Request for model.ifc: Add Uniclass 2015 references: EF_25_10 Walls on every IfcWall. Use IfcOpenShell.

First a look at what the model holds.

```python
import ifcopenshell

model = ifcopenshell.open("model.ifc")
print(model.schema)
print("classifications:", [c.Name for c in model.by_type("IfcClassification")])
for ifc_class in ("IfcDoor", "IfcRoof", "IfcStair", "IfcWall", "IfcWindow"):
    print(ifc_class, len(model.by_type(ifc_class)))
```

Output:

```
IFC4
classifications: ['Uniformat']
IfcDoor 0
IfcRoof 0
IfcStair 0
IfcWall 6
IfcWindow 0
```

```python
import ifcopenshell
import ifcopenshell.api.classification

model = ifcopenshell.open("model.ifc")

system = ifcopenshell.api.classification.add_classification(model, classification="Uniclass 2015")

codes = {
    "IfcWall": ("EF_25_10", "Walls"),
}
for ifc_class, (code, name) in codes.items():
    products = model.by_type(ifc_class)
    ifcopenshell.api.classification.add_reference(
        model, products=products, classification=system, identification=code, name=name
    )
    print(code, len(products))

model.write("model_updated.ifc")
```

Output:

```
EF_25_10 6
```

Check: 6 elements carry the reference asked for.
